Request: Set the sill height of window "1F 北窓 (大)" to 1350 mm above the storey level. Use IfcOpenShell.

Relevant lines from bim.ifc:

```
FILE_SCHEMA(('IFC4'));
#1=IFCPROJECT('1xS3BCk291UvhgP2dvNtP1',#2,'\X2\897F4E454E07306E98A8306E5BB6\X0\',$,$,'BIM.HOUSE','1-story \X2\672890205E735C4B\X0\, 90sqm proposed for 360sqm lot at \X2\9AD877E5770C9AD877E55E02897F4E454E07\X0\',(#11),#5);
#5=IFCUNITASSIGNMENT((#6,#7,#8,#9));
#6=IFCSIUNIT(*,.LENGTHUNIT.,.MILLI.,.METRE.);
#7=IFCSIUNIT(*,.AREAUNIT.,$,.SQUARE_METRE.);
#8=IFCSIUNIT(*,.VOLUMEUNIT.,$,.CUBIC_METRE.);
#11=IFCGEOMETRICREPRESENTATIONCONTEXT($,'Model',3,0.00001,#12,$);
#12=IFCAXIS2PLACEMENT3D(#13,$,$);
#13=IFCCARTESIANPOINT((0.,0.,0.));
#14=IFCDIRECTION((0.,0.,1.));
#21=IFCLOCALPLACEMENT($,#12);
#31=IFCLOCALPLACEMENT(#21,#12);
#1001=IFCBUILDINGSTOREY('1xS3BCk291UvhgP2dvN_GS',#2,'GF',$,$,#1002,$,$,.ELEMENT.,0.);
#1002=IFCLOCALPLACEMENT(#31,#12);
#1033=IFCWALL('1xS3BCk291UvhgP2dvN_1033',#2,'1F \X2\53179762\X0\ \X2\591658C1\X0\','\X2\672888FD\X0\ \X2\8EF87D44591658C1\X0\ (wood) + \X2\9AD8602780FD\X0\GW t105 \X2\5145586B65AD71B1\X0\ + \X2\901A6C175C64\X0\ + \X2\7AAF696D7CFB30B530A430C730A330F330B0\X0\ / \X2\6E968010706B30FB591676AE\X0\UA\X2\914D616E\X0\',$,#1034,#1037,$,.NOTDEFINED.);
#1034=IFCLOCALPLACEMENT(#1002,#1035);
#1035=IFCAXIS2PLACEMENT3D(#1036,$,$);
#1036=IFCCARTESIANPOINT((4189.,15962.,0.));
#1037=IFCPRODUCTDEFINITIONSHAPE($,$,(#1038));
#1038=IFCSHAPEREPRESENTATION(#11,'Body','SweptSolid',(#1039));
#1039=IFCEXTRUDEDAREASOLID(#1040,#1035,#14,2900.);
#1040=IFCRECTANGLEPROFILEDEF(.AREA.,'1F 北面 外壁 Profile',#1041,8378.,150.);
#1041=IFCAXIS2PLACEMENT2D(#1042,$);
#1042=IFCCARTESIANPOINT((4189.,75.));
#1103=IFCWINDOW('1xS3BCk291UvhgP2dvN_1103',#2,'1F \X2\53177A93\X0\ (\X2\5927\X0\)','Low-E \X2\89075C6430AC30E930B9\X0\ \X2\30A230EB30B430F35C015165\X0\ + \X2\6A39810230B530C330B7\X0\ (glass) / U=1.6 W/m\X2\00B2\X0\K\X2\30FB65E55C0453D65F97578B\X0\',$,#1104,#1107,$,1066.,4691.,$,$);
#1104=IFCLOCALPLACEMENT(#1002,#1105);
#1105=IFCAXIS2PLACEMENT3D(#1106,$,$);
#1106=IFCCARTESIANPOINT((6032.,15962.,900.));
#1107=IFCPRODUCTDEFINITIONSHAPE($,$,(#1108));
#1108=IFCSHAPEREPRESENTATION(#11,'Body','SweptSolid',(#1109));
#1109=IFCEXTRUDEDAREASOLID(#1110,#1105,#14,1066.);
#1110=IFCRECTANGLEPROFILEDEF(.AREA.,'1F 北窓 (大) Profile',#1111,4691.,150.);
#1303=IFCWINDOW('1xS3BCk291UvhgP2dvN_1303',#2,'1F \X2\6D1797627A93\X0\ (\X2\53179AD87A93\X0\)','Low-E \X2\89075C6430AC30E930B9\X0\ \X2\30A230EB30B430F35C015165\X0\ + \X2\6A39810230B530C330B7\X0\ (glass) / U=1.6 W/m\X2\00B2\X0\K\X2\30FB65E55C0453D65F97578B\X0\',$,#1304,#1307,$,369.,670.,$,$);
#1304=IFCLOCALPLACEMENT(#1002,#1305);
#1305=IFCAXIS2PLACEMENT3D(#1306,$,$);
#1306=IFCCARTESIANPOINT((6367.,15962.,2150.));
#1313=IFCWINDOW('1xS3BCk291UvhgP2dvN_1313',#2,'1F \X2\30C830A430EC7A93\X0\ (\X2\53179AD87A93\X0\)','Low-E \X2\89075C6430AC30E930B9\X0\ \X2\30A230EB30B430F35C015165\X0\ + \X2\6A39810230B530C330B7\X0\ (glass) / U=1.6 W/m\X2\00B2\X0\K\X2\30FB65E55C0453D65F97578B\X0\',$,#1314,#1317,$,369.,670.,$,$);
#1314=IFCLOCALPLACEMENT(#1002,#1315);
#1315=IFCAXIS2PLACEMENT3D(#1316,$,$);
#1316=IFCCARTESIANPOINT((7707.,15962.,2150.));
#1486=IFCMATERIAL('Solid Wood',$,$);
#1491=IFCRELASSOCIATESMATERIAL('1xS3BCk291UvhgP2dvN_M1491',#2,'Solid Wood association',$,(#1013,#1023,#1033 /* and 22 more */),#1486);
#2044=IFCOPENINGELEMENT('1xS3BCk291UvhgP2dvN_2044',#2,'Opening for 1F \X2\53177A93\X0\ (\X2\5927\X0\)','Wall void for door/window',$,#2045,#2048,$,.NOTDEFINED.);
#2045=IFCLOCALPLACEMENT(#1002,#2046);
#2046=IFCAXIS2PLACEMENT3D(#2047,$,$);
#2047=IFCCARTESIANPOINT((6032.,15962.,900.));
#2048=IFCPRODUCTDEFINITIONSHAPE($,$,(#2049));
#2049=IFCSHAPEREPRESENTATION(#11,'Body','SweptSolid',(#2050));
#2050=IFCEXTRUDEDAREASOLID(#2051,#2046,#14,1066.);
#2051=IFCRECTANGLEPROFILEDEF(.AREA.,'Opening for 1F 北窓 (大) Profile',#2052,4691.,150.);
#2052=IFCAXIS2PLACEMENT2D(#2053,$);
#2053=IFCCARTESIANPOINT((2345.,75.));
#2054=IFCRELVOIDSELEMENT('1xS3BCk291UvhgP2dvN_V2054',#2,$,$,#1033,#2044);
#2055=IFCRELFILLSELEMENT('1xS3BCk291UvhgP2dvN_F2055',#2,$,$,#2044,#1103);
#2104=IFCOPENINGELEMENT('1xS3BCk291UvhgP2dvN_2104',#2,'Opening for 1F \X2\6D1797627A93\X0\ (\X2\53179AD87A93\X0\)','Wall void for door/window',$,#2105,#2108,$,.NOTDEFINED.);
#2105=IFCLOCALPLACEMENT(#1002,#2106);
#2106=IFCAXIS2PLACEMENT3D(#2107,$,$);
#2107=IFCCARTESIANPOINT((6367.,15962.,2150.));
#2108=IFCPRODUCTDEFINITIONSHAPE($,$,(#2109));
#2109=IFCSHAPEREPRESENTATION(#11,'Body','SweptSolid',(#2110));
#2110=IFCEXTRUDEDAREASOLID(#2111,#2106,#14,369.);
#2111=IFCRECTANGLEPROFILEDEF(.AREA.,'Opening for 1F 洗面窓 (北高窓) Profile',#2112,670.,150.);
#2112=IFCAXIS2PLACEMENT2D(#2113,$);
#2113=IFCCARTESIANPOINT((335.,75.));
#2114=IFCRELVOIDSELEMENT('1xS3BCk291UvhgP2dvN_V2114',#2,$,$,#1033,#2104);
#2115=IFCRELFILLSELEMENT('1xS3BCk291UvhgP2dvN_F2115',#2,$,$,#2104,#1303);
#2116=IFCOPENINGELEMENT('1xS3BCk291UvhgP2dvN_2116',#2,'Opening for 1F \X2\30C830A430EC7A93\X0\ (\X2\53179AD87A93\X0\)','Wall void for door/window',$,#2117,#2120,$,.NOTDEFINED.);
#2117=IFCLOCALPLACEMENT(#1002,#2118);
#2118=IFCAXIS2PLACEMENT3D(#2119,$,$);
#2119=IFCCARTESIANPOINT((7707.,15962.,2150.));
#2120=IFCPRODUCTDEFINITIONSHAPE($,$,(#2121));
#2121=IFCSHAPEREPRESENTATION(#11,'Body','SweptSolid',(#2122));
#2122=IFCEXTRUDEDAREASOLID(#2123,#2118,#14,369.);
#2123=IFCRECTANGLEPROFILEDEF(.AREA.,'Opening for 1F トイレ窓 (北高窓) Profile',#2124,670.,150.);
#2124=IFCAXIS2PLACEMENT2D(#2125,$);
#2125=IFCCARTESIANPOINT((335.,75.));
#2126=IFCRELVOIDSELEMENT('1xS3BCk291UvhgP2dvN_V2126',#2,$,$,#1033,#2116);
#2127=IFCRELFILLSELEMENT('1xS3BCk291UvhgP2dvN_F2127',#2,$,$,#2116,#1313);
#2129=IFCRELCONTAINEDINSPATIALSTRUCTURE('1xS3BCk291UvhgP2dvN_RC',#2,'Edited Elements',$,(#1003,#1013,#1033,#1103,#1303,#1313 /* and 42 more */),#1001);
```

```python
import numpy as np
import ifcopenshell
import ifcopenshell.api.geometry
import ifcopenshell.geom
import ifcopenshell.util.element
import ifcopenshell.util.placement
import ifcopenshell.util.shape
import ifcopenshell.util.unit

model = ifcopenshell.open("bim.ifc")
unit_scale = ifcopenshell.util.unit.calculate_unit_scale(model)

window = model.by_guid("1xS3BCk291UvhgP2dvN_1103")
opening = window.FillsVoids[0].RelatingOpeningElement
storey = ifcopenshell.util.element.get_container(window, ifc_class="IfcBuildingStorey")
level = ifcopenshell.util.placement.get_local_placement(storey.ObjectPlacement)[2, 3]

# The opening's origin need not be at the sill, so measure its lowest point.
shape = ifcopenshell.geom.create_shape(ifcopenshell.geom.settings(), opening)
bottom = ifcopenshell.util.shape.get_shape_bottom_elevation(shape, shape.geometry) / unit_scale
dz = level + 1350.0 - bottom

shift = np.array([0.0, 0.0, dz])
# The window is not placed relative to its opening, so move both.
for product in (opening, window):
    matrix = ifcopenshell.util.placement.get_local_placement(product.ObjectPlacement)
    matrix[:3, 3] += shift
    ifcopenshell.api.geometry.edit_object_placement(model, product=product, matrix=matrix, is_si=False)

print(f"moved by {dz * unit_scale:+.3f} m")

model.write("bim-out.ifc")
```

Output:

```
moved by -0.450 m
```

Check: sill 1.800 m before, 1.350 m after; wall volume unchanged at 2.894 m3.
